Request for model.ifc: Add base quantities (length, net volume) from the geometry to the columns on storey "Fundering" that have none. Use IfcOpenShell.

First a look at what the model holds.

```python
import ifcopenshell
import ifcopenshell.util.element
import ifcopenshell.util.unit

model = ifcopenshell.open("model.ifc")
print(model.schema)
for unit_type in ("LENGTHUNIT", "AREAUNIT", "VOLUMEUNIT"):
    print(unit_type, ifcopenshell.util.unit.calculate_unit_scale(model, unit_type))
storey = next(s for s in model.by_type("IfcBuildingStorey") if s.Name == "Fundering")
columns = [e for e in ifcopenshell.util.element.get_decomposition(storey) if e.is_a("IfcColumn")]
for e in sorted(columns, key=lambda e: e.id()):
    print(e.id(), e.is_a(), e.Name, list(ifcopenshell.util.element.get_psets(e, qtos_only=True)), sep=" | ")
```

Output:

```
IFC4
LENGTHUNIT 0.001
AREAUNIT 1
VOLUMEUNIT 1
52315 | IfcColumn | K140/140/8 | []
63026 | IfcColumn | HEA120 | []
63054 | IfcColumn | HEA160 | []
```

```python
import ifcopenshell
import ifcopenshell.api.pset
import ifcopenshell.geom
import ifcopenshell.util.element
import ifcopenshell.util.shape
import ifcopenshell.util.unit

model = ifcopenshell.open("model.ifc")
unit_scale = ifcopenshell.util.unit.calculate_unit_scale(model)
volume_scale = ifcopenshell.util.unit.calculate_unit_scale(model, "VOLUMEUNIT")
settings = ifcopenshell.geom.settings()

storey = next(s for s in model.by_type("IfcBuildingStorey") if s.Name == "Fundering")
columns = [e for e in ifcopenshell.util.element.get_decomposition(storey) if e.is_a("IfcColumn")]

for e in sorted(columns, key=lambda e: e.id()):
    if ifcopenshell.util.element.get_psets(e, qtos_only=True, should_inherit=False):
        continue
    # Geometry comes back in metres, in the element's own axes.
    shape = ifcopenshell.geom.create_shape(settings, e)
    values = {
        "Length": ifcopenshell.util.shape.get_z(shape.geometry) / unit_scale,
        "NetVolume": ifcopenshell.util.shape.get_volume(shape.geometry) / volume_scale,
    }
    qto = ifcopenshell.api.pset.add_qto(model, product=e, name="Qto_ColumnBaseQuantities")
    ifcopenshell.api.pset.edit_qto(model, qto=qto, properties=values)
    print(e.id(), {k: round(v, 3) for k, v in values.items()})

model.write("model_v2.ifc")
```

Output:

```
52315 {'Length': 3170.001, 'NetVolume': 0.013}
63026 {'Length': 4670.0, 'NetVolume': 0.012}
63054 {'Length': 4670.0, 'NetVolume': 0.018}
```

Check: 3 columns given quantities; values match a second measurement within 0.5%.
